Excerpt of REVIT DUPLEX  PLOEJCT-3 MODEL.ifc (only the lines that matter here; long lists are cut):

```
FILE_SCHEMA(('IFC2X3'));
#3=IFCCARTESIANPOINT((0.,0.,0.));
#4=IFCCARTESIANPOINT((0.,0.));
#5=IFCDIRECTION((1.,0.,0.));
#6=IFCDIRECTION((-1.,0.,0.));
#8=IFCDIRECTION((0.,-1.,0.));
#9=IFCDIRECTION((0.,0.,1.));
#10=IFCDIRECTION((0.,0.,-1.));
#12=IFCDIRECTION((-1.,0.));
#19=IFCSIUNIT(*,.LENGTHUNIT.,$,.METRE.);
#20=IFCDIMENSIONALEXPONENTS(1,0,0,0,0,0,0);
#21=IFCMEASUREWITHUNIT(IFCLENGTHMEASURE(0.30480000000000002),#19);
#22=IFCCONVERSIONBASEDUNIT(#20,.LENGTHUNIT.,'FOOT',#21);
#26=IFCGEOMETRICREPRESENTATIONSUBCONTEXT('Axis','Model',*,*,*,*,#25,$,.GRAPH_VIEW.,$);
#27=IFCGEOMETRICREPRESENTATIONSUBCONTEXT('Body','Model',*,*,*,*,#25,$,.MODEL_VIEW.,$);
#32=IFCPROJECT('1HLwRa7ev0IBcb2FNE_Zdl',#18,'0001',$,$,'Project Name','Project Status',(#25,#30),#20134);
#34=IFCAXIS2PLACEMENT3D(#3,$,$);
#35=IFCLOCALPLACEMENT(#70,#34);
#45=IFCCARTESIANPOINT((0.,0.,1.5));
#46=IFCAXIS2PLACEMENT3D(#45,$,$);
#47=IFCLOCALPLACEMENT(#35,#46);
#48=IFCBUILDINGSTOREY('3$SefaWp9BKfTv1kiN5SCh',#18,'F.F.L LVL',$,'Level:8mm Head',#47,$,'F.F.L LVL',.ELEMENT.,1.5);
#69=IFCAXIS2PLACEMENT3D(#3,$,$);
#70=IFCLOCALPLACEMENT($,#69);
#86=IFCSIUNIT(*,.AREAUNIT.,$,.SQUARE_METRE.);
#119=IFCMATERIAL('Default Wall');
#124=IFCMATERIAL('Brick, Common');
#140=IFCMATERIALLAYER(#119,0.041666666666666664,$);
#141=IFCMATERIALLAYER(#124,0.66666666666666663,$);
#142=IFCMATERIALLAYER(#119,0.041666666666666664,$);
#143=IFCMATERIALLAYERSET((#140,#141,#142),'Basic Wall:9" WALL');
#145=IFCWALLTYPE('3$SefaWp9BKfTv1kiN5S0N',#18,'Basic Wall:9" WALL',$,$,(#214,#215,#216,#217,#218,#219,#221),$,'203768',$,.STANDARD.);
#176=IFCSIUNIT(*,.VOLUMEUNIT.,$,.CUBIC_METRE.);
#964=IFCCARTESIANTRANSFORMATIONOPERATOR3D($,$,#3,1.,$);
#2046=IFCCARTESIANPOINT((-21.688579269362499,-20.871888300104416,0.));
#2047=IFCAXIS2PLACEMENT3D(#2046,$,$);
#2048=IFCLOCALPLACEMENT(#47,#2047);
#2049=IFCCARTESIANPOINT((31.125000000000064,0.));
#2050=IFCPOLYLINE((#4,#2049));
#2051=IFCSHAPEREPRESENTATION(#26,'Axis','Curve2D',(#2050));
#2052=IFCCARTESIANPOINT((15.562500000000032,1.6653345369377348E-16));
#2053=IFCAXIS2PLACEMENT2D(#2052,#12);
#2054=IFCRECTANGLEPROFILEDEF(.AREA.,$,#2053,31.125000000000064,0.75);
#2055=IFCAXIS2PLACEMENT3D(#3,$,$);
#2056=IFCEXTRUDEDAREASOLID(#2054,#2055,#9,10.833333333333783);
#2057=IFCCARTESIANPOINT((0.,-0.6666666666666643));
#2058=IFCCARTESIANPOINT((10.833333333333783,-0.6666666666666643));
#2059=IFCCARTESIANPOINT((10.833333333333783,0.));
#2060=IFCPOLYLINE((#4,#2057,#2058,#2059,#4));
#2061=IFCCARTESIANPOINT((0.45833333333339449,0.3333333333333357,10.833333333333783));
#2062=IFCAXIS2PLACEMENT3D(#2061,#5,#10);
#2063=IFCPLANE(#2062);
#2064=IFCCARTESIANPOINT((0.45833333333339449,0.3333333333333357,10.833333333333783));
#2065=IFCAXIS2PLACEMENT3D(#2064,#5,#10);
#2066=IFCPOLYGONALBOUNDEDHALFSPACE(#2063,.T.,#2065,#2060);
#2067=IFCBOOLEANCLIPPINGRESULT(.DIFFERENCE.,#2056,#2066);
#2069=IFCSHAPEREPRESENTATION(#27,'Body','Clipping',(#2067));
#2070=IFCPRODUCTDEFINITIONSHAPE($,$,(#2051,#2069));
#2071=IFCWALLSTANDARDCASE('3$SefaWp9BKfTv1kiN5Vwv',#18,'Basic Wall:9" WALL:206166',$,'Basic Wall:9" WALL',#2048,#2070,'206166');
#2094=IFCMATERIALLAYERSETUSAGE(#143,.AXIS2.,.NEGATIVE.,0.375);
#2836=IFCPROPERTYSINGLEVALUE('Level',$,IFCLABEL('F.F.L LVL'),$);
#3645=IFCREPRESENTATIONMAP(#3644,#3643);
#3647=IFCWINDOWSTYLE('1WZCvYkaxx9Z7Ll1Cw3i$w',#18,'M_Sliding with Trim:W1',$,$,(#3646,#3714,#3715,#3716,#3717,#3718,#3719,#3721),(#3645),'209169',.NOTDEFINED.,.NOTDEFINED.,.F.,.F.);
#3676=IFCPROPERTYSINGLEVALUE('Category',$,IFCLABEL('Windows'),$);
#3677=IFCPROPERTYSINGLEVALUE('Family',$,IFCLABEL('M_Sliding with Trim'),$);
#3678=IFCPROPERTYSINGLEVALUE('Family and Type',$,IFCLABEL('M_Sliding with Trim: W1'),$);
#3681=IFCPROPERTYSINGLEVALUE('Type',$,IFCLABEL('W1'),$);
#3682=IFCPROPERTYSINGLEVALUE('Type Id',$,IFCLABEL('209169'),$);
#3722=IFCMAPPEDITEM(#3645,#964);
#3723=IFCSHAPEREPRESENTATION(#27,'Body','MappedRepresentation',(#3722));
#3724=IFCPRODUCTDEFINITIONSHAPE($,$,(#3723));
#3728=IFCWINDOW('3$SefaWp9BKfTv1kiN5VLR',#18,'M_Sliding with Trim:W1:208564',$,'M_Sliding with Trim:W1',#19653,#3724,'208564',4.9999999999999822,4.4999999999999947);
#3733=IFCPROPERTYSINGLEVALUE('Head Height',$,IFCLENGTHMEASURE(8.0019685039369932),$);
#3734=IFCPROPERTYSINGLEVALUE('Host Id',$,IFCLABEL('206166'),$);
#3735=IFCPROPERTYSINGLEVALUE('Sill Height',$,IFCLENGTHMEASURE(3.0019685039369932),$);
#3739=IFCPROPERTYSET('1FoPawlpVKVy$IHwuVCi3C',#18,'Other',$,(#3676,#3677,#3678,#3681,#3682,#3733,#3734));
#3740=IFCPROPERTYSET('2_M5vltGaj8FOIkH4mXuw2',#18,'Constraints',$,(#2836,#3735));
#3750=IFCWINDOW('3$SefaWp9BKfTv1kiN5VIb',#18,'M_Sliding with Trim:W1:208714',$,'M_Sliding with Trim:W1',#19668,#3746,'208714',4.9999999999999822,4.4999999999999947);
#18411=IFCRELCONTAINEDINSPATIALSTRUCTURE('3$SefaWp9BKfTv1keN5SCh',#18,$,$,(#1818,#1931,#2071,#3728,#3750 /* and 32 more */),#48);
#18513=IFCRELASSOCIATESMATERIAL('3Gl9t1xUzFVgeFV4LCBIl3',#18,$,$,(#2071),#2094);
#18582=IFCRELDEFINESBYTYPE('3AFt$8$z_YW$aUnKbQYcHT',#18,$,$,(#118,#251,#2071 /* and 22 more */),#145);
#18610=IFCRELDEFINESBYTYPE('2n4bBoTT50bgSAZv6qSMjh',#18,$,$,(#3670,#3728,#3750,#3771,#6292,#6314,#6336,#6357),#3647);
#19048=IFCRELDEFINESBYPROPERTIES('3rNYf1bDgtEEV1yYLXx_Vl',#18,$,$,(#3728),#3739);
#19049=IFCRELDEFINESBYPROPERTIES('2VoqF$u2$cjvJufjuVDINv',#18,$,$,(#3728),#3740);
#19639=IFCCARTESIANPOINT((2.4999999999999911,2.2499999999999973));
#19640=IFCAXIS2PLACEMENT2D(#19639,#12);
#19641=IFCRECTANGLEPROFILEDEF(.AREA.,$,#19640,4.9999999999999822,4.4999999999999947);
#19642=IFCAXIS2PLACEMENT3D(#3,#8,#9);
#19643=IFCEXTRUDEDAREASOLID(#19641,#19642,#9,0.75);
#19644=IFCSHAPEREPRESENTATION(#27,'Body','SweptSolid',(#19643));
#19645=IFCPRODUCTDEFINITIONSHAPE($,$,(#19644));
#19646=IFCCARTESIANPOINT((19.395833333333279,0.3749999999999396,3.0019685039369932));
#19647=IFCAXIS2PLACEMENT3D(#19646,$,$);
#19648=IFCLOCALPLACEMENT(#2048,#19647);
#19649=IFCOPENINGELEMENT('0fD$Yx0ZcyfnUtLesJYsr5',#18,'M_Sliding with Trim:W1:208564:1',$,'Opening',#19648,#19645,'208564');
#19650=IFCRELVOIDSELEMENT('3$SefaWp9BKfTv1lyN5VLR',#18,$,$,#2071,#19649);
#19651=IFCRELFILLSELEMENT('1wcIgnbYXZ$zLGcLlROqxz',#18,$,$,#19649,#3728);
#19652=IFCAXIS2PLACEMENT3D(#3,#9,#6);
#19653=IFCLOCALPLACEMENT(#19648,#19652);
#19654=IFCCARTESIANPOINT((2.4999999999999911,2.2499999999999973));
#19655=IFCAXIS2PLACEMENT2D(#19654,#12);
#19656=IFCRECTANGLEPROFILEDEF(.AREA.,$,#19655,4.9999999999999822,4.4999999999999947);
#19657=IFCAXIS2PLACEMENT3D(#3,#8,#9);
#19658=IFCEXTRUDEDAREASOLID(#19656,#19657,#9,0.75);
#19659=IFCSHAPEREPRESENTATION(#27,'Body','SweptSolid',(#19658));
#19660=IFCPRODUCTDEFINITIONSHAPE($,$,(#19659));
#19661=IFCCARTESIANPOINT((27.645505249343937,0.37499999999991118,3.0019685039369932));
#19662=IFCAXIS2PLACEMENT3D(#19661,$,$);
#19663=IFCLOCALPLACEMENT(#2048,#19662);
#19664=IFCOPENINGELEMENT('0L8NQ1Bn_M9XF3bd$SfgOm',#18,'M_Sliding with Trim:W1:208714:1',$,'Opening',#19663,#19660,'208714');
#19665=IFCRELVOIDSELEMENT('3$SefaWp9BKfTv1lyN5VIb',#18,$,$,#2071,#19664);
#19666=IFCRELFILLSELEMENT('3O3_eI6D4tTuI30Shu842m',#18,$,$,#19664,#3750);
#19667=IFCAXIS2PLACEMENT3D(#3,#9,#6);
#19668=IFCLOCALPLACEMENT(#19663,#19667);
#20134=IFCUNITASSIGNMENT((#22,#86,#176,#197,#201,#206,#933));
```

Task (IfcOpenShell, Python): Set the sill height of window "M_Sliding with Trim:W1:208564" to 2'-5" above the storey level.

```python
import numpy as np
import ifcopenshell
import ifcopenshell.api.geometry
import ifcopenshell.api.pset
import ifcopenshell.geom
import ifcopenshell.util.element
import ifcopenshell.util.placement
import ifcopenshell.util.shape
import ifcopenshell.util.unit

model = ifcopenshell.open("REVIT DUPLEX  PLOEJCT-3 MODEL.ifc")
unit_scale = ifcopenshell.util.unit.calculate_unit_scale(model)

window = model.by_guid("3$SefaWp9BKfTv1kiN5VLR")
opening = window.FillsVoids[0].RelatingOpeningElement
storey = ifcopenshell.util.element.get_container(window, ifc_class="IfcBuildingStorey")
level = ifcopenshell.util.placement.get_local_placement(storey.ObjectPlacement)[2, 3]

# The opening's origin need not be at the sill, so measure its lowest point.
shape = ifcopenshell.geom.create_shape(ifcopenshell.geom.settings(), opening)
bottom = ifcopenshell.util.shape.get_shape_bottom_elevation(shape, shape.geometry) / unit_scale
dz = level + 29 * 0.0254 / unit_scale - bottom

shift = np.array([0.0, 0.0, dz])
# The window is placed relative to its opening, so it follows when the opening moves.
matrix = ifcopenshell.util.placement.get_local_placement(opening.ObjectPlacement)
matrix[:3, 3] += shift
ifcopenshell.api.geometry.edit_object_placement(
    model, product=opening, matrix=matrix, is_si=False, should_transform_children=True
)

# Keep the stored heights in step.
pset = model.by_id(ifcopenshell.util.element.get_pset(window, "Other", should_inherit=False)["id"])
ifcopenshell.api.pset.edit_pset(model, pset=pset, properties={
    "Head Height": model.create_entity("IfcLengthMeasure", ifcopenshell.util.element.get_pset(window, "Other", "Head Height") + dz),
})
pset = model.by_id(ifcopenshell.util.element.get_pset(window, "Constraints", should_inherit=False)["id"])
ifcopenshell.api.pset.edit_pset(model, pset=pset, properties={
    "Sill Height": model.create_entity("IfcLengthMeasure", ifcopenshell.util.element.get_pset(window, "Constraints", "Sill Height") + dz),
})

print(f"moved by {dz * unit_scale:+.3f} m")

model.write("REVIT DUPLEX  PLOEJCT-3 MODEL_rev.ifc")
```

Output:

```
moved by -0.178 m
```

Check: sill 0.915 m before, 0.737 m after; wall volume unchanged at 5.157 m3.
